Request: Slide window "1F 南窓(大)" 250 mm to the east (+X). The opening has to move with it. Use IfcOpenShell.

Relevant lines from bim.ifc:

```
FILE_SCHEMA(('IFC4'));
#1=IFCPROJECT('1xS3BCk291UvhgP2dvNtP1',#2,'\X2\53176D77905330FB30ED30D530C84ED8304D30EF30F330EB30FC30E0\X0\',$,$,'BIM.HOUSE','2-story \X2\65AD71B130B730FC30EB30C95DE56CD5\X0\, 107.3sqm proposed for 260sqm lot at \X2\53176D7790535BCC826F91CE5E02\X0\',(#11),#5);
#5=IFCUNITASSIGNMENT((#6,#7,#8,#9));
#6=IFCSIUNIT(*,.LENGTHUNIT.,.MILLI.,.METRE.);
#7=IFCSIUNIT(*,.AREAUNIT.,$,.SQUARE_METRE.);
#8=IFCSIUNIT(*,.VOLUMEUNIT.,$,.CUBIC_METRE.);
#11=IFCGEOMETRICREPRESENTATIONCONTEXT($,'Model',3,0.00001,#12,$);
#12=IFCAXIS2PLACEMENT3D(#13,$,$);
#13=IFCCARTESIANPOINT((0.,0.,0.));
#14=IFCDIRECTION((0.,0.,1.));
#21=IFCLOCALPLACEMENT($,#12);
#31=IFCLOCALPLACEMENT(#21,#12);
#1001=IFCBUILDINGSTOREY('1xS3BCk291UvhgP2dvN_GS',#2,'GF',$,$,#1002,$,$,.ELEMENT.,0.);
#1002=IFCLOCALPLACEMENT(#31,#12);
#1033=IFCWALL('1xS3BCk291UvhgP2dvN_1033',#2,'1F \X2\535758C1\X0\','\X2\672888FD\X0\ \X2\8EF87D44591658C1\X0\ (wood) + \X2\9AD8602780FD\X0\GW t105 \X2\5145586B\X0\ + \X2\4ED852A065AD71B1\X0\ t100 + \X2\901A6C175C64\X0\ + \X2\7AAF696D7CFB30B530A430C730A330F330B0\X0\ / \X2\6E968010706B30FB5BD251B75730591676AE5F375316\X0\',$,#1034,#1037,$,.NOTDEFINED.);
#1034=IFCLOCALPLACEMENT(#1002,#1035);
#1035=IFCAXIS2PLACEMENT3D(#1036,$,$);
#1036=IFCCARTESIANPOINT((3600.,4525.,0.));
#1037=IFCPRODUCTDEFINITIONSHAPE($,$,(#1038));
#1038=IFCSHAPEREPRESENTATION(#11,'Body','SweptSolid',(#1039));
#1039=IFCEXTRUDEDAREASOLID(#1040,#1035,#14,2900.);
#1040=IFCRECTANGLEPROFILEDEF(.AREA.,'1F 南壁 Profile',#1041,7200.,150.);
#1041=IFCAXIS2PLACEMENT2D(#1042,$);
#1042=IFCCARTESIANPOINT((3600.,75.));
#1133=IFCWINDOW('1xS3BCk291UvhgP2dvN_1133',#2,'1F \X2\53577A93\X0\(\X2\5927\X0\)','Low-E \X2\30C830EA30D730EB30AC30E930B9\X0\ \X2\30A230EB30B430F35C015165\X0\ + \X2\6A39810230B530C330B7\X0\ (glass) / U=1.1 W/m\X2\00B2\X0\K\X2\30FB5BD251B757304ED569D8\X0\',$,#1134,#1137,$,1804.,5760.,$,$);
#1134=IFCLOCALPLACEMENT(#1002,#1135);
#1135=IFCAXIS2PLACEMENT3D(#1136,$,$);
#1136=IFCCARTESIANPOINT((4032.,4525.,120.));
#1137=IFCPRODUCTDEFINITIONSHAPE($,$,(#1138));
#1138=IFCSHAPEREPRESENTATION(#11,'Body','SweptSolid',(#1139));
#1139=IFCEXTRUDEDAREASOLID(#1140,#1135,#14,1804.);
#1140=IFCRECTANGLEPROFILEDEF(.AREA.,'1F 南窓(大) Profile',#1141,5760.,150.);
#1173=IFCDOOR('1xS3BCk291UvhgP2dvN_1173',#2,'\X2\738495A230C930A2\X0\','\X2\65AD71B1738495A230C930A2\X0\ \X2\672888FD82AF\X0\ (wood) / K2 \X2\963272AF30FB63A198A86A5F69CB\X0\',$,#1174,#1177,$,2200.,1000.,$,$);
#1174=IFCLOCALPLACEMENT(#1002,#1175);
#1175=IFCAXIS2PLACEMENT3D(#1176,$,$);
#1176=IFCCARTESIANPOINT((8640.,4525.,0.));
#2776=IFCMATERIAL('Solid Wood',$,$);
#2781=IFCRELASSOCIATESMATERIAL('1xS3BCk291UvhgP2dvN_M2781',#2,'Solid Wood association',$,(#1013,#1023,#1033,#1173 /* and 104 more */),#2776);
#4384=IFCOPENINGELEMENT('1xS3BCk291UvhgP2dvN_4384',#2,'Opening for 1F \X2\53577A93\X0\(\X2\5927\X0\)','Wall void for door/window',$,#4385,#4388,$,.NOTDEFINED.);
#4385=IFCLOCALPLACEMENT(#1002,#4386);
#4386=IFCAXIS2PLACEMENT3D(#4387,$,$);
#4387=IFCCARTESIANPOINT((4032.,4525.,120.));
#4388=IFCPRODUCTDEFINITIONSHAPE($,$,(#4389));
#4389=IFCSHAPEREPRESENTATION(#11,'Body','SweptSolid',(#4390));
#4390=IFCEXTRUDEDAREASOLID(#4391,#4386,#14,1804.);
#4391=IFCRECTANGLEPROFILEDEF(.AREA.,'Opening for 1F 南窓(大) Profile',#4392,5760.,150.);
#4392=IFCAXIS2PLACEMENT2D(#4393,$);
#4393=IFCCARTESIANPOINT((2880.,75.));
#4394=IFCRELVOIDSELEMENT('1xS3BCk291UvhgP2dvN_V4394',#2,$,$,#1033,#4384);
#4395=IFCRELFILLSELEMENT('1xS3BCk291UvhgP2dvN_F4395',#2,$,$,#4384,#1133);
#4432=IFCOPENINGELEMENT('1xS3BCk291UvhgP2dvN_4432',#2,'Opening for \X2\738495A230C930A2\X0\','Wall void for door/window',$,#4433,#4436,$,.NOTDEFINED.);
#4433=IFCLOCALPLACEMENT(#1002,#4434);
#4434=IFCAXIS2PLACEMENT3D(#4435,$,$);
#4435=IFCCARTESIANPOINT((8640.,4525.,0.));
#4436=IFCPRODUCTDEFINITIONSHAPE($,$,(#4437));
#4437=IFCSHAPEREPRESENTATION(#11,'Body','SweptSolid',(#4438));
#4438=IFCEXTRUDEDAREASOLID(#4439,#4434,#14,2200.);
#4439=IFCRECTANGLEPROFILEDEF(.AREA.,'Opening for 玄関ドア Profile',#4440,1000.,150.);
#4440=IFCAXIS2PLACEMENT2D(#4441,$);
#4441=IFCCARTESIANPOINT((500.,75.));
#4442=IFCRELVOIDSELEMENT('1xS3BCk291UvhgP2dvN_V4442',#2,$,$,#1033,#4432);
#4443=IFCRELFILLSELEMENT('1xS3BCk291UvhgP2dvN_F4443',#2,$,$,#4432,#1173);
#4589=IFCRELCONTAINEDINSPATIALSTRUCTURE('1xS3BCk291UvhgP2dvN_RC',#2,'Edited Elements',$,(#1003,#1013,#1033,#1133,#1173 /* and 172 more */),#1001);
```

```python
import ifcopenshell
import ifcopenshell.api.geometry
import ifcopenshell.util.placement
import ifcopenshell.util.unit

model = ifcopenshell.open("bim.ifc")
unit_scale = ifcopenshell.util.unit.calculate_unit_scale(model)

window = model.by_guid("1xS3BCk291UvhgP2dvN_1133")
opening = window.FillsVoids[0].RelatingOpeningElement
wall = opening.VoidsElements[0].RelatingBuildingElement

wall_matrix = ifcopenshell.util.placement.get_local_placement(wall.ObjectPlacement)
shift = wall_matrix[:3, 0] * 0.25 / unit_scale
before = ifcopenshell.util.placement.get_local_placement(window.ObjectPlacement)[:3, 3].copy()

# The window is not placed relative to its opening, so move both.
for product in (opening, window):
    matrix = ifcopenshell.util.placement.get_local_placement(product.ObjectPlacement)
    matrix[:3, 3] += shift
    ifcopenshell.api.geometry.edit_object_placement(model, product=product, matrix=matrix, is_si=False)

after = ifcopenshell.util.placement.get_local_placement(window.ObjectPlacement)[:3, 3]
print("window moved by", (after - before).round(3) + 0.0)

model.write("bim_v2.ifc")
```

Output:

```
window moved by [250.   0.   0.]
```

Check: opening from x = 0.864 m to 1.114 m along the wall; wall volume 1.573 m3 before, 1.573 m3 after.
